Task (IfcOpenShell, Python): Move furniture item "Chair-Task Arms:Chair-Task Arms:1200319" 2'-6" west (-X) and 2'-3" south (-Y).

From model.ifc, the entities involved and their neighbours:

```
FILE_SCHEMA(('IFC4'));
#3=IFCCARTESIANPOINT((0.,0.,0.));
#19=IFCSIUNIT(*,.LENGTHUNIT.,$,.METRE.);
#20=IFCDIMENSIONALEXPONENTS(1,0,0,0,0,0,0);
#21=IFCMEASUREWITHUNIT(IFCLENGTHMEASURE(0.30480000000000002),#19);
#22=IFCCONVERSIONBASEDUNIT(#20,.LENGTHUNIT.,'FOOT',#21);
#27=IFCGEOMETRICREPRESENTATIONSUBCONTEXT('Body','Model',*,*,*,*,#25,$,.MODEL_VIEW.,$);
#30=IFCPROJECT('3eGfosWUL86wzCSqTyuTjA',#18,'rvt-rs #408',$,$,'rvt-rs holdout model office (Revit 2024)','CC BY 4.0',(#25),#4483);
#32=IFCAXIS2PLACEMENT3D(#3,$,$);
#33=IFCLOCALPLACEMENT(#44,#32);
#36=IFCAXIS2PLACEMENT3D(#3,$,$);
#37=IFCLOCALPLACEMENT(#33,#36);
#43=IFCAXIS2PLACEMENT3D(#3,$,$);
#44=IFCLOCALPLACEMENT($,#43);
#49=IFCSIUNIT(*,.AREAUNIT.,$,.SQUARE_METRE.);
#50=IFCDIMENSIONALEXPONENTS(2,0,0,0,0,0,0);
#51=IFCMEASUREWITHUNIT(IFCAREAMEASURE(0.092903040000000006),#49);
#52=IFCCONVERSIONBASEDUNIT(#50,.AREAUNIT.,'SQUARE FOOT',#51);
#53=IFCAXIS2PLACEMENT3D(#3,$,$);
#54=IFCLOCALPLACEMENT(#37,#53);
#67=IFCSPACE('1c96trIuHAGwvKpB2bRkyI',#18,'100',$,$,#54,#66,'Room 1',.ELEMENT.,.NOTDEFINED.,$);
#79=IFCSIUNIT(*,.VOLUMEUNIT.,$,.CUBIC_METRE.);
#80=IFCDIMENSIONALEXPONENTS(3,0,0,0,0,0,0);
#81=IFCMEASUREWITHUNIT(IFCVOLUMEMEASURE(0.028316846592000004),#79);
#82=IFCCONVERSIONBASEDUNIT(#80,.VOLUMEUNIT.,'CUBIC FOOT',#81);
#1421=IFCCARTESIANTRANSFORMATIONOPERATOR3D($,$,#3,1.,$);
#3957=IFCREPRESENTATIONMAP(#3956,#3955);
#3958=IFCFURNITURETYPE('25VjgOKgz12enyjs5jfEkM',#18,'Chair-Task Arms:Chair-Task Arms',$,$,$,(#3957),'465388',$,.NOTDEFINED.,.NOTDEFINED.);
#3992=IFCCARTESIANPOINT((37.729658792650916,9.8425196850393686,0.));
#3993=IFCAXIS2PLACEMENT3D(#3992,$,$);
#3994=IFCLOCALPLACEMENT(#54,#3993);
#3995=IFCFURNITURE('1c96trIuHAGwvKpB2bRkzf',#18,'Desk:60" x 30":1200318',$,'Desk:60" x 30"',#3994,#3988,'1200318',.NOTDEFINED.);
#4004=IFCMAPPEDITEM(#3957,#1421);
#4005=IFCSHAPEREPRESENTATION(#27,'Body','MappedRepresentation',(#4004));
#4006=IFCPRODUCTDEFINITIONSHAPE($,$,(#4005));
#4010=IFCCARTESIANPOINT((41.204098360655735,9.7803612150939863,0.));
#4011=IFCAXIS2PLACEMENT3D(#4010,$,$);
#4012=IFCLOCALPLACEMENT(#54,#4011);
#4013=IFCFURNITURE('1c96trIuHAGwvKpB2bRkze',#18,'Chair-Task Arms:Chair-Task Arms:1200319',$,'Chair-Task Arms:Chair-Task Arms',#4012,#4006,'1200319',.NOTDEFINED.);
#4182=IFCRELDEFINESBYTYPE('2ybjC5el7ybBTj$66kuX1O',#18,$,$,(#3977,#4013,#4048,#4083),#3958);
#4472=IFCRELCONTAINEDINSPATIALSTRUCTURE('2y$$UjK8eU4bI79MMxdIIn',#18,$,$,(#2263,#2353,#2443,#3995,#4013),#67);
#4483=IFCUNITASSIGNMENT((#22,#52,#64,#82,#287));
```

```python
import ifcopenshell
import ifcopenshell.api.geometry
import ifcopenshell.util.placement
import ifcopenshell.util.unit

model = ifcopenshell.open("model.ifc")
unit_scale = ifcopenshell.util.unit.calculate_unit_scale(model)

item = model.by_guid("1c96trIuHAGwvKpB2bRkze")
matrix = ifcopenshell.util.placement.get_local_placement(item.ObjectPlacement)
matrix[0, 3] -= 30 * 0.0254 / unit_scale
matrix[1, 3] -= 27 * 0.0254 / unit_scale
ifcopenshell.api.geometry.edit_object_placement(model, product=item, matrix=matrix, is_si=False)

print(ifcopenshell.util.placement.get_local_placement(item.ObjectPlacement).round(3) + 0.0)

model.write("model-out.ifc")
```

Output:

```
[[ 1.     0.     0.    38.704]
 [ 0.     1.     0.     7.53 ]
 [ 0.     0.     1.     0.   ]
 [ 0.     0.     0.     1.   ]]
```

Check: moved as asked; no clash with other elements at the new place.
